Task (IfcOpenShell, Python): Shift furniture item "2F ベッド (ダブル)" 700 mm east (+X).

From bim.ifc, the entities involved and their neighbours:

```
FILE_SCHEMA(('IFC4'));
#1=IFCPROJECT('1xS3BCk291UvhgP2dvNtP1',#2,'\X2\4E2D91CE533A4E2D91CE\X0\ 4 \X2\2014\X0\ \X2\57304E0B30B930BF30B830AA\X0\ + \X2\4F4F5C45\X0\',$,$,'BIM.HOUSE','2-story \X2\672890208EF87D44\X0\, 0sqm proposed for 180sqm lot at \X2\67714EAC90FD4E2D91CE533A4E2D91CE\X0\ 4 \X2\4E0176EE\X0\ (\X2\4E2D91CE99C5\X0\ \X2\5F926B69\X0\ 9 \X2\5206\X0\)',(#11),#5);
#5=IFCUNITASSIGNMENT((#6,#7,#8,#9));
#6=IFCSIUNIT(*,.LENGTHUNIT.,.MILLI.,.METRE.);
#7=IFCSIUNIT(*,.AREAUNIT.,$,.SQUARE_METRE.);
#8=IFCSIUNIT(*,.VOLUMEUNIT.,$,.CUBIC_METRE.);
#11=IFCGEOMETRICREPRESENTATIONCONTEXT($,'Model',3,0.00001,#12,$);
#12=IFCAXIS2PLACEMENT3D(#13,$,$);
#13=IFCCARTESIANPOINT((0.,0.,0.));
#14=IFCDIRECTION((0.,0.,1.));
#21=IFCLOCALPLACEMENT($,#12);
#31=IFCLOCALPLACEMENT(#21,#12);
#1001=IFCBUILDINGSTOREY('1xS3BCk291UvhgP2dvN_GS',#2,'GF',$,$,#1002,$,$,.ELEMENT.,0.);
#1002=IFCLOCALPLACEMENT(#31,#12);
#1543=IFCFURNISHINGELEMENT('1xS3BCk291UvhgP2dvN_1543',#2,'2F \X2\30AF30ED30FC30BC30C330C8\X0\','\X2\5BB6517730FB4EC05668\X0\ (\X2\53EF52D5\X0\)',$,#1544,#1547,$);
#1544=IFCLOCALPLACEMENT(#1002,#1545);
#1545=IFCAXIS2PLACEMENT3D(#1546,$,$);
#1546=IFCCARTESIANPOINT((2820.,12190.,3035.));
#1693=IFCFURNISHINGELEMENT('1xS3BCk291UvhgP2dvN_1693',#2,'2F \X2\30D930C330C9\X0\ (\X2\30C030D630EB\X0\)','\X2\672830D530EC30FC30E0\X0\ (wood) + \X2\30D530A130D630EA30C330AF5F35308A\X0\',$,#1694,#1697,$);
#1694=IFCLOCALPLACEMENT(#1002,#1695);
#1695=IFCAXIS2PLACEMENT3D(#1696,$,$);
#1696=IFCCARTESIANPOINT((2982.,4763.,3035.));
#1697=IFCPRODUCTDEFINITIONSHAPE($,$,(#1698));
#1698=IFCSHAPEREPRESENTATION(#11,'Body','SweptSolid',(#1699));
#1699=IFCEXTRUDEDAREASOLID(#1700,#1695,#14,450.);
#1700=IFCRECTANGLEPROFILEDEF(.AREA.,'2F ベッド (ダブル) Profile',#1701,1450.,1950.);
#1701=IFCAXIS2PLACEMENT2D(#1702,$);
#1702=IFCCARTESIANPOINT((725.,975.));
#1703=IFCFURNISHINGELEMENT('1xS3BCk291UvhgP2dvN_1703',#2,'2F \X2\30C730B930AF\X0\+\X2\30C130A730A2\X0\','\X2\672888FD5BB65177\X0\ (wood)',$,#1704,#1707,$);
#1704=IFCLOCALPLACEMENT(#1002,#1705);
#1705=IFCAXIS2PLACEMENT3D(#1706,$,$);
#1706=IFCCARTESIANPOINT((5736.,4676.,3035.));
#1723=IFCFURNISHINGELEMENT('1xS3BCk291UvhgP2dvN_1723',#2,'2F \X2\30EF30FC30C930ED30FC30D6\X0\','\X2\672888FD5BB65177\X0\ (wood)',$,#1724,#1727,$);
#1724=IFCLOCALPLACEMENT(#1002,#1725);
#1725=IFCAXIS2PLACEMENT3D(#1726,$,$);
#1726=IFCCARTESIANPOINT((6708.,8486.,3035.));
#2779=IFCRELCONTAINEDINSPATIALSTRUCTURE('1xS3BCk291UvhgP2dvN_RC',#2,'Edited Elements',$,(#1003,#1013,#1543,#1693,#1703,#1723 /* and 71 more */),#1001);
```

```python
import ifcopenshell
import ifcopenshell.api.geometry
import ifcopenshell.util.placement

model = ifcopenshell.open("bim.ifc")

item = model.by_id(1693)
matrix = ifcopenshell.util.placement.get_local_placement(item.ObjectPlacement)
matrix[0, 3] += 700.0
ifcopenshell.api.geometry.edit_object_placement(model, product=item, matrix=matrix, is_si=False)

print(ifcopenshell.util.placement.get_local_placement(item.ObjectPlacement).round(3) + 0.0)

model.write("bim-out.ifc")
```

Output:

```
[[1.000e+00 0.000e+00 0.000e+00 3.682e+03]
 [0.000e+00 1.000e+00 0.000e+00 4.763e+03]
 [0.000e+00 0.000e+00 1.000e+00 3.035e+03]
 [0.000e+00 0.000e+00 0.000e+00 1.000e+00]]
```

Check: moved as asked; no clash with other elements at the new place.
